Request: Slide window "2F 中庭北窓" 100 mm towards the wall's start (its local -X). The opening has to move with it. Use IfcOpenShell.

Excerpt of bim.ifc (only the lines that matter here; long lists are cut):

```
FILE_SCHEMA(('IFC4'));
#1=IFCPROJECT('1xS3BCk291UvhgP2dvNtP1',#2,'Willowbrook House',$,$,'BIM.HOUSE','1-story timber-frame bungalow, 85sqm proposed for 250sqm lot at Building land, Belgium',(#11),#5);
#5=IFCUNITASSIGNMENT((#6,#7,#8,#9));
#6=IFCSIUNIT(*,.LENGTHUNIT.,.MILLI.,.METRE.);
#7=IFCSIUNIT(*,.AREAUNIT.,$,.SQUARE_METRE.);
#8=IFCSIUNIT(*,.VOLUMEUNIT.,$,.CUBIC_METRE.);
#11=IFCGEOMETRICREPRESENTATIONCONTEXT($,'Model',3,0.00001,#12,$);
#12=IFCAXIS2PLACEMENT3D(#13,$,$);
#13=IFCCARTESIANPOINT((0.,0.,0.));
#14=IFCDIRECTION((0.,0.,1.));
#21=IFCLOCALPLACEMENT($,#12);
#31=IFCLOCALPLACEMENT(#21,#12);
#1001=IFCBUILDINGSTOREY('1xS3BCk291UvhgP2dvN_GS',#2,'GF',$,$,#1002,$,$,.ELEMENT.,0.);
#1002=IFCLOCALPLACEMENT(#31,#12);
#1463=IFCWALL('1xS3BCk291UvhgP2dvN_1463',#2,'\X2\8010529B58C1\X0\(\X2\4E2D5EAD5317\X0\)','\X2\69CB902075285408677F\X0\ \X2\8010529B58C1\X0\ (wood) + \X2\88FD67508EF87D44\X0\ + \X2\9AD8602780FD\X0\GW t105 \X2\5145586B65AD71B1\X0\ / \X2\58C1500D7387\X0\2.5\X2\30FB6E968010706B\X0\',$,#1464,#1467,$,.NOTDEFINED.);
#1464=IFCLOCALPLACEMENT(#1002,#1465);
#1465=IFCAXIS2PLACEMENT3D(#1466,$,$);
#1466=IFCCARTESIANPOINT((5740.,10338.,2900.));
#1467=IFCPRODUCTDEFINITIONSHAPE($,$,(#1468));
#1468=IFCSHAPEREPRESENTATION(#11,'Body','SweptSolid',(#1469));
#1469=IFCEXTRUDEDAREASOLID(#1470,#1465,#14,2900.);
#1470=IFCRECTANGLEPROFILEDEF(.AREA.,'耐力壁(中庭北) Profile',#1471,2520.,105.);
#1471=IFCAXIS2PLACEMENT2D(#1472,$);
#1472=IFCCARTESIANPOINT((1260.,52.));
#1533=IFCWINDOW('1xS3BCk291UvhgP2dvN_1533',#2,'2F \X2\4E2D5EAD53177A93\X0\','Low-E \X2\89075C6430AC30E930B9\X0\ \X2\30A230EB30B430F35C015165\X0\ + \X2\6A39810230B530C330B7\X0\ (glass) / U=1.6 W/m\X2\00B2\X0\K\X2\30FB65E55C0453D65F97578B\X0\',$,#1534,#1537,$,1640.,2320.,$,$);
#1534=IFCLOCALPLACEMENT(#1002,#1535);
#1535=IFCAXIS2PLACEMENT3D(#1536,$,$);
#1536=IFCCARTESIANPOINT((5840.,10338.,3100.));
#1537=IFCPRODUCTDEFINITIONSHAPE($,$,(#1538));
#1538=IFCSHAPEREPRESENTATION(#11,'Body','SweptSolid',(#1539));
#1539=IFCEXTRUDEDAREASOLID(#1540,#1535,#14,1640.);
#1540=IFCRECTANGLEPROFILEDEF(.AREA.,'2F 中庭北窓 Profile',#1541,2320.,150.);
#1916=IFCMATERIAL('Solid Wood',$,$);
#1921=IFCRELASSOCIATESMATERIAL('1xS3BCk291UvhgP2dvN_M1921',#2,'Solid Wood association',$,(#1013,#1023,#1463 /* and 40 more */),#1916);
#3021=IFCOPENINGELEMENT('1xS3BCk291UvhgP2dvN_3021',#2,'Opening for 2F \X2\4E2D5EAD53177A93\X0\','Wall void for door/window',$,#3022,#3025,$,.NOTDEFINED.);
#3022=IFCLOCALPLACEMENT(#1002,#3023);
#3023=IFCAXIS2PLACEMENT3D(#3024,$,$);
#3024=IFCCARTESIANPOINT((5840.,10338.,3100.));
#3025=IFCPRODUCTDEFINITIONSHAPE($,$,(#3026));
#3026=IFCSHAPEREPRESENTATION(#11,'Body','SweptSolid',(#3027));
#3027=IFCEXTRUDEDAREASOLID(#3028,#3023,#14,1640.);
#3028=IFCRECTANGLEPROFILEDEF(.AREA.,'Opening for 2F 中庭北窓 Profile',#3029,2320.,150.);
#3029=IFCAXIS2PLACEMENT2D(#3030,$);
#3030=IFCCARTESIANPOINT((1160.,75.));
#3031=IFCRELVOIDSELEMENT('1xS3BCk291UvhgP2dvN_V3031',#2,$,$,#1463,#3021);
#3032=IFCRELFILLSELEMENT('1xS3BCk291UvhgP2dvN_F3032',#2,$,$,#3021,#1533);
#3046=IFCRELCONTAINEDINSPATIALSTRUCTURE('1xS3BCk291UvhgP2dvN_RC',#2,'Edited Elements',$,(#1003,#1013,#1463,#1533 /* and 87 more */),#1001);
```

```python
import ifcopenshell
import ifcopenshell.api.geometry
import ifcopenshell.util.placement

model = ifcopenshell.open("bim.ifc")

window = model.by_guid("1xS3BCk291UvhgP2dvN_1533")
opening = window.FillsVoids[0].RelatingOpeningElement
wall = opening.VoidsElements[0].RelatingBuildingElement

wall_matrix = ifcopenshell.util.placement.get_local_placement(wall.ObjectPlacement)
shift = wall_matrix[:3, 0] * -100.0
before = ifcopenshell.util.placement.get_local_placement(window.ObjectPlacement)[:3, 3].copy()

# The window is not placed relative to its opening, so move both.
for product in (opening, window):
    matrix = ifcopenshell.util.placement.get_local_placement(product.ObjectPlacement)
    matrix[:3, 3] += shift
    ifcopenshell.api.geometry.edit_object_placement(model, product=product, matrix=matrix, is_si=False)

after = ifcopenshell.util.placement.get_local_placement(window.ObjectPlacement)[:3, 3]
print("window moved by", (after - before).round(3) + 0.0)

model.write("bim_rev.ifc")
```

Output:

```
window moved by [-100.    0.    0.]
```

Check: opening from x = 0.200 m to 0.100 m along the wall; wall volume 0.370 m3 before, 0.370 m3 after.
